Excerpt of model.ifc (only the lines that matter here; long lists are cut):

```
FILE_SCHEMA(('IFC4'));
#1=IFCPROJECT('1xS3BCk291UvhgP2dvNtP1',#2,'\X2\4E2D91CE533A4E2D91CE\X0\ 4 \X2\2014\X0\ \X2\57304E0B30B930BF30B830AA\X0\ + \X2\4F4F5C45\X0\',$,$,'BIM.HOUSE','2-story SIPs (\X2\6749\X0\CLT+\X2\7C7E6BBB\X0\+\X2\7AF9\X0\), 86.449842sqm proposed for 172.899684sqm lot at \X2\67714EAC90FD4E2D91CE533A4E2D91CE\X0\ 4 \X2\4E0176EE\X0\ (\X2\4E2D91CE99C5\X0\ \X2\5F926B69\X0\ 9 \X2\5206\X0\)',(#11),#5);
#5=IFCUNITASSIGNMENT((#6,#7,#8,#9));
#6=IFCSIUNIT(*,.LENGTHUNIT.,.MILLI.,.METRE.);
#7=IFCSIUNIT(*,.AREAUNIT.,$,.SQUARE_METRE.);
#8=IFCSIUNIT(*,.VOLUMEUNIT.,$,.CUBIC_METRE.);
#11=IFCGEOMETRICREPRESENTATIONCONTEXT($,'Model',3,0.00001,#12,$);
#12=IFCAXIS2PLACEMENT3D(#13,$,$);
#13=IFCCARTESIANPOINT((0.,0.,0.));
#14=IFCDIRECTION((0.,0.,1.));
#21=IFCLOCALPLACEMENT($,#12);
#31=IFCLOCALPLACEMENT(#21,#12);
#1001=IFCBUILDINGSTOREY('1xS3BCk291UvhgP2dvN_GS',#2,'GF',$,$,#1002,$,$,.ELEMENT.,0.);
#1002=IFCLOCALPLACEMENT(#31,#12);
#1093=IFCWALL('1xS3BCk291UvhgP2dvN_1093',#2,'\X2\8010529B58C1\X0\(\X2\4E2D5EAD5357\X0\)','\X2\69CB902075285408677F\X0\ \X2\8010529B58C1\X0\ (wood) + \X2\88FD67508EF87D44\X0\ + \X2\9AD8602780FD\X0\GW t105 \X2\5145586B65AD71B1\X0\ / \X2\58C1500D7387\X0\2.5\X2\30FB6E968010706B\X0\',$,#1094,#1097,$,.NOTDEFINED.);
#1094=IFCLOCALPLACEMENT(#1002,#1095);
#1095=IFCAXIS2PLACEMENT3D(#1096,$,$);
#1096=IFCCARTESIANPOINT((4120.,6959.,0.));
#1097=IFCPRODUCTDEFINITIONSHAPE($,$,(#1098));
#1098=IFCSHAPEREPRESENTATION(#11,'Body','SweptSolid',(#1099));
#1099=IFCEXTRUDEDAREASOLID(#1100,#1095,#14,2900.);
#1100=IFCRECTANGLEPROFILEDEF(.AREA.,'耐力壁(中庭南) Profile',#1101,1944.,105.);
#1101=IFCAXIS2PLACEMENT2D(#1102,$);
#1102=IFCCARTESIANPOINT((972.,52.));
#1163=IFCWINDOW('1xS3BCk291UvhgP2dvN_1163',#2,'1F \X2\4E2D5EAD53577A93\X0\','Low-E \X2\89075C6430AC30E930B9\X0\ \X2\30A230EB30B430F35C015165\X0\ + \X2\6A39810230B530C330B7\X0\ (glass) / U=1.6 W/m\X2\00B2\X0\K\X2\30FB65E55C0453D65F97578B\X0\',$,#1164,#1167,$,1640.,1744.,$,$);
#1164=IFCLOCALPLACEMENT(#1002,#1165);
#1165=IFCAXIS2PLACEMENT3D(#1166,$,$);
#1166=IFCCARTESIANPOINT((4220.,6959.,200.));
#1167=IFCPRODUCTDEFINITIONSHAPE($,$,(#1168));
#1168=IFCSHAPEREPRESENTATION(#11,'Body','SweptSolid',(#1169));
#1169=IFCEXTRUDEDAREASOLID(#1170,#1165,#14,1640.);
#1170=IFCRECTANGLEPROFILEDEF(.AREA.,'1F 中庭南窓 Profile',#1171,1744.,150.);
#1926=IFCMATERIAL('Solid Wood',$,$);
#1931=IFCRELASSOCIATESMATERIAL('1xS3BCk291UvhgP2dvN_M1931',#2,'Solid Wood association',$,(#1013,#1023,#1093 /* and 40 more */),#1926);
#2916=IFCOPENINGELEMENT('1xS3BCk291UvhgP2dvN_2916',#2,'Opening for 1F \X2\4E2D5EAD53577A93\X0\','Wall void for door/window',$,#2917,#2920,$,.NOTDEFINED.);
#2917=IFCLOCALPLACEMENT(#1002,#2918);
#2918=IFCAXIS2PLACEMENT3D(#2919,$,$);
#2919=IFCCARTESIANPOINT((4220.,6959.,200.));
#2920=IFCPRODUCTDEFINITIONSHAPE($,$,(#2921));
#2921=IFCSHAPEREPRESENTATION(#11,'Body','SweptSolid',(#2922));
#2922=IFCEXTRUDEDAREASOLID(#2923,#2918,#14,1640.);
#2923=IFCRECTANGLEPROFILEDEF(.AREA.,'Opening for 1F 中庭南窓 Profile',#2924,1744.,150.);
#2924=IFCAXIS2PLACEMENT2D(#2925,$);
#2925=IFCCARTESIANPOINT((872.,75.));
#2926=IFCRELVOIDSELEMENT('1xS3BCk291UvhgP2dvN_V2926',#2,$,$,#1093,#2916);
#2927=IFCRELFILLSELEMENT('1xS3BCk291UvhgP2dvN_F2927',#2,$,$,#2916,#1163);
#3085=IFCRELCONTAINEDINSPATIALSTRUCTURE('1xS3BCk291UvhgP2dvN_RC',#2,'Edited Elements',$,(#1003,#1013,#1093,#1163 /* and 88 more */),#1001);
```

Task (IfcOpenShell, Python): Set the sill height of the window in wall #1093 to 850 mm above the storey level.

```python
import numpy as np
import ifcopenshell
import ifcopenshell.api.geometry
import ifcopenshell.geom
import ifcopenshell.util.element
import ifcopenshell.util.placement
import ifcopenshell.util.shape
import ifcopenshell.util.unit

model = ifcopenshell.open("model.ifc")
unit_scale = ifcopenshell.util.unit.calculate_unit_scale(model)

window = model.by_id(1163)
opening = window.FillsVoids[0].RelatingOpeningElement
storey = ifcopenshell.util.element.get_container(window, ifc_class="IfcBuildingStorey")
level = ifcopenshell.util.placement.get_local_placement(storey.ObjectPlacement)[2, 3]

# The opening's origin need not be at the sill, so measure its lowest point.
shape = ifcopenshell.geom.create_shape(ifcopenshell.geom.settings(), opening)
bottom = ifcopenshell.util.shape.get_shape_bottom_elevation(shape, shape.geometry) / unit_scale
dz = level + 0.85 / unit_scale - bottom

shift = np.array([0.0, 0.0, dz])
# The window is not placed relative to its opening, so move both.
for product in (opening, window):
    matrix = ifcopenshell.util.placement.get_local_placement(product.ObjectPlacement)
    matrix[:3, 3] += shift
    ifcopenshell.api.geometry.edit_object_placement(model, product=product, matrix=matrix, is_si=False)

print(f"moved by {dz * unit_scale:+.3f} m")

model.write("model_rev.ifc")
```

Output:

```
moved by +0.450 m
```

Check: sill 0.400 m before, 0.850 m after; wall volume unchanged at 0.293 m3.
